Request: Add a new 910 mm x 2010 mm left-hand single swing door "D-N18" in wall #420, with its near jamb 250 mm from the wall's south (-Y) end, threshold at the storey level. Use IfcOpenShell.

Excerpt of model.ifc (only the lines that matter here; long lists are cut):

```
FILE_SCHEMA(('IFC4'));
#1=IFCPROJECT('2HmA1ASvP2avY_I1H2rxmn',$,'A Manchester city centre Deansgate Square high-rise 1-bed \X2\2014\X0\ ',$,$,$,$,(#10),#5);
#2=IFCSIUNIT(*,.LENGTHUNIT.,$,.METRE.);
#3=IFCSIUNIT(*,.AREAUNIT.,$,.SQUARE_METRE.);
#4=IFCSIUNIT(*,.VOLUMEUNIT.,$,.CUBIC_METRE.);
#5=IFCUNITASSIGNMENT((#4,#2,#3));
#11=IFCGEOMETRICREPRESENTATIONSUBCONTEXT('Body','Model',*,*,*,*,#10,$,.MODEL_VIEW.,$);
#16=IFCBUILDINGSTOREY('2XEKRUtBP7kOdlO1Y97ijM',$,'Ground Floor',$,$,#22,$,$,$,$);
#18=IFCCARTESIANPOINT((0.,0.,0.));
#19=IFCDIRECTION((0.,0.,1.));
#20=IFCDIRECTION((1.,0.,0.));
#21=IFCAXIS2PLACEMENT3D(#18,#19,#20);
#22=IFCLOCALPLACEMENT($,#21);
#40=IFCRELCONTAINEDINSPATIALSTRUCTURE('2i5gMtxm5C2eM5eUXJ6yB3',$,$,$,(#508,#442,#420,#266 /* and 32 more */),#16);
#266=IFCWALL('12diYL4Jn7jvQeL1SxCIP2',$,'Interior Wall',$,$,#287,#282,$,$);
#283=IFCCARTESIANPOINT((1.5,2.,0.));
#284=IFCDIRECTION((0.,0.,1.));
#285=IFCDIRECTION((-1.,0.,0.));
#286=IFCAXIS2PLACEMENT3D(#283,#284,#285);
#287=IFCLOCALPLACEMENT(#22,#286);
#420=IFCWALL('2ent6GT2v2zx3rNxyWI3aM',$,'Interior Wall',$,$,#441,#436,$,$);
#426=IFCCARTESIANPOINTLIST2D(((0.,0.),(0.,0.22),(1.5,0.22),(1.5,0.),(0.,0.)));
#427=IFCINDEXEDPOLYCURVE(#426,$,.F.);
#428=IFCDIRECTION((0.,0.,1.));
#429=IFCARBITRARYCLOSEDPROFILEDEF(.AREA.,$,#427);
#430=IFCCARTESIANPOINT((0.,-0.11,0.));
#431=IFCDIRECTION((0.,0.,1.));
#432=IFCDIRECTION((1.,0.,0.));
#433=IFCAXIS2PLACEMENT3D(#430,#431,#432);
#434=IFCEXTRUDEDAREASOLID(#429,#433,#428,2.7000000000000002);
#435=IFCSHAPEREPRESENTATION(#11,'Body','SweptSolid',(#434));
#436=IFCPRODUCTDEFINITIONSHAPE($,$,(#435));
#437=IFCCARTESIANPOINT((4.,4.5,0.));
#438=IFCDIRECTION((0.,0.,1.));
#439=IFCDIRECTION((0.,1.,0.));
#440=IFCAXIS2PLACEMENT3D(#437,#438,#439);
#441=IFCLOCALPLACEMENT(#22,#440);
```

```python
import numpy as np
import ifcopenshell
import ifcopenshell.api.feature
import ifcopenshell.api.geometry
import ifcopenshell.api.root
import ifcopenshell.api.spatial
import ifcopenshell.geom
import ifcopenshell.util.element
import ifcopenshell.util.placement
import ifcopenshell.util.representation
import ifcopenshell.util.shape
import ifcopenshell.util.unit

model = ifcopenshell.open("model.ifc")
unit_scale = ifcopenshell.util.unit.calculate_unit_scale(model)
settings = ifcopenshell.geom.settings()


def volume(element):
    """Net volume in cubic metres, openings subtracted."""
    shape = ifcopenshell.geom.create_shape(settings, element)
    return ifcopenshell.util.shape.get_volume(shape.geometry)


wall = model.by_guid("2ent6GT2v2zx3rNxyWI3aM")
storey = ifcopenshell.util.element.get_container(wall, ifc_class="IfcBuildingStorey")
context = ifcopenshell.util.representation.get_context(model, "Model", "Body", "MODEL_VIEW")
before = volume(wall)

width, height, from_end, sill = 0.91, 2.01, 0.25, 0.0  # metres

# The wall runs along its own X axis, and the end named is its -X end.
wall_shape = ifcopenshell.geom.create_shape(settings, wall)
x, y, z = ifcopenshell.util.shape.get_vertices(wall_shape.geometry).T
start = x.min() + from_end
face, thickness = float(y.min()), float(y.max() - y.min())
wall_matrix = ifcopenshell.util.placement.get_local_placement(wall.ObjectPlacement)
level = ifcopenshell.util.placement.get_local_placement(storey.ObjectPlacement)[2, 3]


def in_wall(x, y):
    """Placement at x, y metres in the wall's axes, at sill height."""
    matrix = wall_matrix.copy()
    matrix[:, 3] = wall_matrix @ np.array([x / unit_scale, y / unit_scale, 0.0, 1.0])
    matrix[2, 3] = level + sill / unit_scale
    return matrix


# Opening: a box that overshoots both wall faces by 50 mm.
opening = ifcopenshell.api.root.create_entity(model, ifc_class="IfcOpeningElement", predefined_type="OPENING")
box = ifcopenshell.api.geometry.add_wall_representation(
    model, context=context, length=width, height=height, thickness=thickness + 0.1
)
ifcopenshell.api.geometry.assign_representation(model, product=opening, representation=box)
ifcopenshell.api.geometry.edit_object_placement(model, product=opening, matrix=in_wall(start, face - 0.05), is_si=False)
ifcopenshell.api.feature.add_feature(model, feature=opening, element=wall)

door = ifcopenshell.api.root.create_entity(model, ifc_class="IfcDoor", name="D-N18", predefined_type="DOOR")
door.OverallWidth, door.OverallHeight = width / unit_scale, height / unit_scale
door.OperationType = "SINGLE_SWING_LEFT"
body = ifcopenshell.api.geometry.add_door_representation(
    model,
    context=context,
    overall_width=door.OverallWidth,
    overall_height=door.OverallHeight,
    operation_type="SINGLE_SWING_LEFT",
    lining_properties={"LiningDepth": thickness / unit_scale, "ThresholdDepth": thickness / unit_scale},
)
ifcopenshell.api.geometry.assign_representation(model, product=door, representation=body)
ifcopenshell.api.spatial.assign_container(model, products=[door], relating_structure=storey)
ifcopenshell.api.feature.add_filling(model, opening=opening, element=door)

# The lining spans the wall, so the door starts at the wall face.
ifcopenshell.api.geometry.edit_object_placement(model, product=door, matrix=in_wall(start, face), is_si=False)

after = volume(wall)

print(f"wall volume {before:.3f} -> {after:.3f} m3")

model.write("model_rev.ifc")
```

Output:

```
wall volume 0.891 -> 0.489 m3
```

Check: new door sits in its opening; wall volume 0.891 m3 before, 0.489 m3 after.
